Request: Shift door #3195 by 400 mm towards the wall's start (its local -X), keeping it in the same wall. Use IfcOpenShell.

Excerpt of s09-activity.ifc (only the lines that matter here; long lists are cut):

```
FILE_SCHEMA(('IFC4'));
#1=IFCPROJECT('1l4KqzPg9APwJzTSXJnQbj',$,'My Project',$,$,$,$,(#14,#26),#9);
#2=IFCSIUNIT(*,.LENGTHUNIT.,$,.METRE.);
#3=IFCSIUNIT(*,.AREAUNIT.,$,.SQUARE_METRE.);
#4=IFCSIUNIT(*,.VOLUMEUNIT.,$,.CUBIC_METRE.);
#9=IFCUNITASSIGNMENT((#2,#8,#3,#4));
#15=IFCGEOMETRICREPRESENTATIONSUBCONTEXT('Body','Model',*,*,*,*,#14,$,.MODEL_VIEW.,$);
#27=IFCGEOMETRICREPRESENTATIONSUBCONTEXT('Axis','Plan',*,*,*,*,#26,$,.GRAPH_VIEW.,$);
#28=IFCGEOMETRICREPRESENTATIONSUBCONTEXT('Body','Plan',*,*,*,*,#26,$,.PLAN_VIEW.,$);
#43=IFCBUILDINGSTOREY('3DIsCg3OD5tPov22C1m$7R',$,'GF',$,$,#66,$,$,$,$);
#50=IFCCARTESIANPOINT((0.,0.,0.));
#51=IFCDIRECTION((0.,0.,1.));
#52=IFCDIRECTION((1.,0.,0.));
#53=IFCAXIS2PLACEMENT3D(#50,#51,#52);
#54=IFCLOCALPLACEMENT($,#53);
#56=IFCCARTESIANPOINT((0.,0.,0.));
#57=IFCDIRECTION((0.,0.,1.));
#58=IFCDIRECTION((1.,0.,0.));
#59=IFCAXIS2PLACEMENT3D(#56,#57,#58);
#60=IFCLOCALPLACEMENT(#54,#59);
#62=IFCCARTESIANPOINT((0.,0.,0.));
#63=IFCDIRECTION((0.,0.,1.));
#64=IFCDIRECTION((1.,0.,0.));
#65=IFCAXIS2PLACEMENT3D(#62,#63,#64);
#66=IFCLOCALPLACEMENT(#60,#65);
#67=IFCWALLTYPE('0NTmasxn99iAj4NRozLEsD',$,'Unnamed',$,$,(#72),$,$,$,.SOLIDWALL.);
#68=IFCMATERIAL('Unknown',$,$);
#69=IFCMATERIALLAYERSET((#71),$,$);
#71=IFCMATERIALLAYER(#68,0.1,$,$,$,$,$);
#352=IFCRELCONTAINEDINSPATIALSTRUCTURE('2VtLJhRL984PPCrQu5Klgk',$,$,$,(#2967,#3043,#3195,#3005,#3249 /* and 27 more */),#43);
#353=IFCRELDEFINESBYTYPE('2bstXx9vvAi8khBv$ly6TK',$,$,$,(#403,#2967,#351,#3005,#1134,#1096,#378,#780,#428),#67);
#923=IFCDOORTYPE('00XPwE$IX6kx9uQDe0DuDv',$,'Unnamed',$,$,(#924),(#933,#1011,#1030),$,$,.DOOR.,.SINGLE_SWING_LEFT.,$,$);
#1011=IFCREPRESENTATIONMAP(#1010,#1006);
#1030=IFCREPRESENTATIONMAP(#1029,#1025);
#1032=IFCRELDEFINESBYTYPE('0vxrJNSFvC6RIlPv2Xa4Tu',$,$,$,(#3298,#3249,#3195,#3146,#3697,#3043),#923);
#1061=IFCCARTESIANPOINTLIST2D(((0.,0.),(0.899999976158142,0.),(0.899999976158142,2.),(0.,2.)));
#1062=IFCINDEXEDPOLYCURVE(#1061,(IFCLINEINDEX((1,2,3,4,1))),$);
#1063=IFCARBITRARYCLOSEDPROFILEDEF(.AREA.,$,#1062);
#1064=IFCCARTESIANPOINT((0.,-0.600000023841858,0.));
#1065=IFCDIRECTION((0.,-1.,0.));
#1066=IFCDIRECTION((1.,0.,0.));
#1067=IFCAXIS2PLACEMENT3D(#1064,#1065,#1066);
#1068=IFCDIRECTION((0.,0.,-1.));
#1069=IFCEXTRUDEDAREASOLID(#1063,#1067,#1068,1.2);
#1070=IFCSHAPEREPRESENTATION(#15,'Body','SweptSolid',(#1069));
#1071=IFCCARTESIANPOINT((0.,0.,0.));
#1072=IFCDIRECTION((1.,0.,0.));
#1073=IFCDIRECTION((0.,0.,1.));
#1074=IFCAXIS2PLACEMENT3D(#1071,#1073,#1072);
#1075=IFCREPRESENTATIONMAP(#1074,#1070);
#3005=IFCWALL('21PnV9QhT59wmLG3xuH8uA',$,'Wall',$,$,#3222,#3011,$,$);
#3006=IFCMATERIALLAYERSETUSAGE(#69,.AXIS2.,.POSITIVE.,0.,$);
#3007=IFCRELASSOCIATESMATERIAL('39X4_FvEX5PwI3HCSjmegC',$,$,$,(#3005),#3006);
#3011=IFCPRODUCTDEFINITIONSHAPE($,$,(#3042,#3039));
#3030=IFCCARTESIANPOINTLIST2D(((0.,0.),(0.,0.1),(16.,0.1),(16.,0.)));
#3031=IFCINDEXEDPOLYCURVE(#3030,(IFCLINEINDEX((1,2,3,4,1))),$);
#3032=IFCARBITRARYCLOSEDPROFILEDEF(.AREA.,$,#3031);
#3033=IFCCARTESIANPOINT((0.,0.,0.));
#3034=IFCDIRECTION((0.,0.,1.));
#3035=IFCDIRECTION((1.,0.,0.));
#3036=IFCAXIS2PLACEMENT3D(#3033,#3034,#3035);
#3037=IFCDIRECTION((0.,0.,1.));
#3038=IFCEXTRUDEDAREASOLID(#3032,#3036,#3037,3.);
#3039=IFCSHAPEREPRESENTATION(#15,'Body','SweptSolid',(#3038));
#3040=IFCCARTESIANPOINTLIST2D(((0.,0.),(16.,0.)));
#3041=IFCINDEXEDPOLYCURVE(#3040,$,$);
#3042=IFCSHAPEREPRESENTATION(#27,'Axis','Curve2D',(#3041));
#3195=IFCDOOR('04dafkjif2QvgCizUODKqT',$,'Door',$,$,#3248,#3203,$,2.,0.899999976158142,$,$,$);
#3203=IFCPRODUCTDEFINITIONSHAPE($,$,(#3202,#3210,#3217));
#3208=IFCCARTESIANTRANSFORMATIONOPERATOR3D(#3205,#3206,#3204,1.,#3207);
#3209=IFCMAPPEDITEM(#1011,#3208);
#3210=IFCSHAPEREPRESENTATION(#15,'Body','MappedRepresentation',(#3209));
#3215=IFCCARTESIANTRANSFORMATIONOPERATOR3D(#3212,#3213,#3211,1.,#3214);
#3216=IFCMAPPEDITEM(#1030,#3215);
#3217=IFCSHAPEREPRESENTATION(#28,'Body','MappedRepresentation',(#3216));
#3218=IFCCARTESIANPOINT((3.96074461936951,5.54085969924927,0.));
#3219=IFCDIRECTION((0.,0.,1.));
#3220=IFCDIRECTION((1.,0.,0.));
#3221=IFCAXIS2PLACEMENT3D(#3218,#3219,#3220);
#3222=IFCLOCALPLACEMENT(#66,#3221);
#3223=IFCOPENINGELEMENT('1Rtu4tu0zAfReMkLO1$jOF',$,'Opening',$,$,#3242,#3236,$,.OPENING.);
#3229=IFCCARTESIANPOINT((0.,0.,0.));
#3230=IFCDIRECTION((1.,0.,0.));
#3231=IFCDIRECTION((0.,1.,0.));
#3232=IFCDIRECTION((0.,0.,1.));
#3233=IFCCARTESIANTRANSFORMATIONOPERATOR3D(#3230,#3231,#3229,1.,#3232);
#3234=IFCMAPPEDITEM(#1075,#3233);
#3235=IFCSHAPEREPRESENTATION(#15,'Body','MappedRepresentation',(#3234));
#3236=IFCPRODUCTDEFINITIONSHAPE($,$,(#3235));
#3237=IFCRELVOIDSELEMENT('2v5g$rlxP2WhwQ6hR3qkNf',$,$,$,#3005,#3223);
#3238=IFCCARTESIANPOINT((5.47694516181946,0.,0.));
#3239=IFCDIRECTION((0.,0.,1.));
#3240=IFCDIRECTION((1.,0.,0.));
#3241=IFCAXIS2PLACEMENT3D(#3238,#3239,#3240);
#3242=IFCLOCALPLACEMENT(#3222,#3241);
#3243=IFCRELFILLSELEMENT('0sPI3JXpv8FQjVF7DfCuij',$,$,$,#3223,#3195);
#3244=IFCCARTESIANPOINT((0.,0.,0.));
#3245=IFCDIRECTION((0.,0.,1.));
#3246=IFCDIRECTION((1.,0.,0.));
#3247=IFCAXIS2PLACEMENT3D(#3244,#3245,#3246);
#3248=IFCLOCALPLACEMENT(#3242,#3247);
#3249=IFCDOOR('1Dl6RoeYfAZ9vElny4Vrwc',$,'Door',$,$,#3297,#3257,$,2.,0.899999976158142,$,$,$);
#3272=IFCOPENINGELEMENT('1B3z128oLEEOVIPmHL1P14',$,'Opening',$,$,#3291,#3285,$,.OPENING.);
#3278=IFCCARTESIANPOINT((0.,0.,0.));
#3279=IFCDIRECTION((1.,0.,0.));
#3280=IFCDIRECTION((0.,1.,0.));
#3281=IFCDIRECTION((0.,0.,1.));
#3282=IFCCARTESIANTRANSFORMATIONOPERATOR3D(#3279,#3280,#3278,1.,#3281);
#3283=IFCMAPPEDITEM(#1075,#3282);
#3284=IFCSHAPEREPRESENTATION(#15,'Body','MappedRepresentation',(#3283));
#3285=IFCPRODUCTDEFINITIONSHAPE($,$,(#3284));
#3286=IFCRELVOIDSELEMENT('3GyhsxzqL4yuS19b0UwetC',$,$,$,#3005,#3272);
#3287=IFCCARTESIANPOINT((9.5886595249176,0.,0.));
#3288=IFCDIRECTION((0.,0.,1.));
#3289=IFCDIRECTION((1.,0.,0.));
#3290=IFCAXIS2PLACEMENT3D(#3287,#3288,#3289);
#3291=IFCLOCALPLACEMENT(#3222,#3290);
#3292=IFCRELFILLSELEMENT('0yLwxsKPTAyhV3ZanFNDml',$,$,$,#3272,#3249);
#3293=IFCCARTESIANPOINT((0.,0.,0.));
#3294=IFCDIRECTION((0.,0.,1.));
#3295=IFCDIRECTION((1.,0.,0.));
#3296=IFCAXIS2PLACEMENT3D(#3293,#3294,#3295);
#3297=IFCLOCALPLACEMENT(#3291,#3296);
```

```python
import ifcopenshell
import ifcopenshell.api.geometry
import ifcopenshell.util.placement
import ifcopenshell.util.unit

model = ifcopenshell.open("s09-activity.ifc")
unit_scale = ifcopenshell.util.unit.calculate_unit_scale(model)

door = model.by_guid("04dafkjif2QvgCizUODKqT")
opening = door.FillsVoids[0].RelatingOpeningElement
wall = opening.VoidsElements[0].RelatingBuildingElement

wall_matrix = ifcopenshell.util.placement.get_local_placement(wall.ObjectPlacement)
shift = wall_matrix[:3, 0] * -0.4 / unit_scale
before = ifcopenshell.util.placement.get_local_placement(door.ObjectPlacement)[:3, 3].copy()

# The door is placed relative to its opening, so it follows when the opening moves.
matrix = ifcopenshell.util.placement.get_local_placement(opening.ObjectPlacement)
matrix[:3, 3] += shift
ifcopenshell.api.geometry.edit_object_placement(
    model, product=opening, matrix=matrix, is_si=False, should_transform_children=True
)

after = ifcopenshell.util.placement.get_local_placement(door.ObjectPlacement)[:3, 3]
print("door moved by", (after - before).round(3) + 0.0)

model.write("s09-activity_v2.ifc")
```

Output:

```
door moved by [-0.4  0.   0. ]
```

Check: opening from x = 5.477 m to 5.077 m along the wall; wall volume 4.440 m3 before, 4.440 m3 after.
